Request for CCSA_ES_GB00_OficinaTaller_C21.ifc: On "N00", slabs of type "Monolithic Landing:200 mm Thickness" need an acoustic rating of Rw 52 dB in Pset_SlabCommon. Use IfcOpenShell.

First a look at what the model holds.

```python
import ifcopenshell
import ifcopenshell.util.element

model = ifcopenshell.open("CCSA_ES_GB00_OficinaTaller_C21.ifc")
print(model.schema)
storey = next(s for s in model.by_type("IfcBuildingStorey") if s.Name == "N00")
slabs = [e for e in ifcopenshell.util.element.get_decomposition(storey) if e.is_a("IfcSlab")]
seen = {}
for e in slabs:
    element_type = ifcopenshell.util.element.get_type(e)
    key = (element_type.Name if element_type != e and element_type else None, ifcopenshell.util.element.get_pset(e, "Pset_SlabCommon", "AcousticRating"))
    seen[key] = seen.get(key, 0) + 1
for (name, value), count in sorted(seen.items(), key=str):
    print(count, "x", name, "|", value)
```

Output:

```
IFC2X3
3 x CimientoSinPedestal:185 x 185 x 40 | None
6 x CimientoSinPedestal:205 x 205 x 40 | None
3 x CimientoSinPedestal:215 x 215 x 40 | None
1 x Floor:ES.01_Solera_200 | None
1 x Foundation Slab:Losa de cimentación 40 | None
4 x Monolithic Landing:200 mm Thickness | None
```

```python
import ifcopenshell
import ifcopenshell.api.pset
import ifcopenshell.util.element

model = ifcopenshell.open("CCSA_ES_GB00_OficinaTaller_C21.ifc")

storey = next(s for s in model.by_type("IfcBuildingStorey") if s.Name == "N00")
slabs = [e for e in ifcopenshell.util.element.get_decomposition(storey) if e.is_a("IfcSlab")]

count = 0
for e in slabs:
    element_type = ifcopenshell.util.element.get_type(e)
    if element_type in (None, e) or element_type.Name != "Monolithic Landing:200 mm Thickness":
        continue
    # add_pset returns the element's existing set when there is one.
    pset = ifcopenshell.api.pset.add_pset(model, product=e, name="Pset_SlabCommon")
    ifcopenshell.api.pset.edit_pset(model, pset=pset, properties={"AcousticRating": "Rw 52 dB"})
    count += 1

print(count, "slabs updated")

model.write("CCSA_ES_GB00_OficinaTaller_C21-out.ifc")
```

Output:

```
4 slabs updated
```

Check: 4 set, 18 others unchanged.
